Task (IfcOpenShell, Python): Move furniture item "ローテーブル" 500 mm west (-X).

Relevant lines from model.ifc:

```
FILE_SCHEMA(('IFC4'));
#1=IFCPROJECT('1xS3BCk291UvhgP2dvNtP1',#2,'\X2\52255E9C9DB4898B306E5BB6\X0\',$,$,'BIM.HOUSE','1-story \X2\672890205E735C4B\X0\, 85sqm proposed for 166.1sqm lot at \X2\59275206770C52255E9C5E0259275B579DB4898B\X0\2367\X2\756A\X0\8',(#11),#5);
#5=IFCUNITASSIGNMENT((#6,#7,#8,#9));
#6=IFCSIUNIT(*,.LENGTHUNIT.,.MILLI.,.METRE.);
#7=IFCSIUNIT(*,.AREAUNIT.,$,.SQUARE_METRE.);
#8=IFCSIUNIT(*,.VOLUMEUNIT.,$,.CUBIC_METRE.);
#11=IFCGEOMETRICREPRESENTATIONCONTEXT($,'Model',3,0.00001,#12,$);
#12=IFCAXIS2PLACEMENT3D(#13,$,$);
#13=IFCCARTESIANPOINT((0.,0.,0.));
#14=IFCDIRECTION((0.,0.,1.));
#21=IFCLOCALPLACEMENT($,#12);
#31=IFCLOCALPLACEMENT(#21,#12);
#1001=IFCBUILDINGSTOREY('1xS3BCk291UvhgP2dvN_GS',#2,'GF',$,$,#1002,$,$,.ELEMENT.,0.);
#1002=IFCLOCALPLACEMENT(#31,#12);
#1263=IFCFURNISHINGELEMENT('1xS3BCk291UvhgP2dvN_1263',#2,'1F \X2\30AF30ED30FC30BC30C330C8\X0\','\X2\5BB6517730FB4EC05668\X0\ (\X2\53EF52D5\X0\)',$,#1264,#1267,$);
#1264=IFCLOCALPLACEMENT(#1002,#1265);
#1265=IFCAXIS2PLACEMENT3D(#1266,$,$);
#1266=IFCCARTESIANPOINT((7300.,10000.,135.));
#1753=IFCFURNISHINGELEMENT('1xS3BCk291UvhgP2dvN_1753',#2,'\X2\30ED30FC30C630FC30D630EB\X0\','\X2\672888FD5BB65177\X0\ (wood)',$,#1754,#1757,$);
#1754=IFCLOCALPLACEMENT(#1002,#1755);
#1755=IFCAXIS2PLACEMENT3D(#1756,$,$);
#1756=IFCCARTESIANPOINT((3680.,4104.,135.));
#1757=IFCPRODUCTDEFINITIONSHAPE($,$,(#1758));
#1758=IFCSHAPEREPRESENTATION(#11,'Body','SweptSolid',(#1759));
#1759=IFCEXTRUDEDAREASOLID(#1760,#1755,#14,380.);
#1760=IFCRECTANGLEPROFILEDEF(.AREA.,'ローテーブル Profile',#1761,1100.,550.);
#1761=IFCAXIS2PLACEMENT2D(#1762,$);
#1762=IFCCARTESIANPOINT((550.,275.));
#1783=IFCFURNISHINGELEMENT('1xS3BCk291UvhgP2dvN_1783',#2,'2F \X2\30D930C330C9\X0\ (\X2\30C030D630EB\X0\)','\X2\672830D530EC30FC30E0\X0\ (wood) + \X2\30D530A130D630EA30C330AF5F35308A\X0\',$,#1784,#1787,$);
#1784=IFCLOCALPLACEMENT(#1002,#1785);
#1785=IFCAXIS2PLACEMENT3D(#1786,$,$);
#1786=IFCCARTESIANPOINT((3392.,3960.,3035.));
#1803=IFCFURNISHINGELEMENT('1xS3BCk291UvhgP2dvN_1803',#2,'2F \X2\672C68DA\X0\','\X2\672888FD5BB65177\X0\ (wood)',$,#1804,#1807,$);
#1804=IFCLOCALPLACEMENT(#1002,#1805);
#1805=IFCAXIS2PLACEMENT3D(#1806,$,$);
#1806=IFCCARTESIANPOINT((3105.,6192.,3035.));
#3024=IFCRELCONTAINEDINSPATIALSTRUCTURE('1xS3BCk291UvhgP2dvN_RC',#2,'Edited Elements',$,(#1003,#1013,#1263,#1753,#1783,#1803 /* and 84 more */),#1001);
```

```python
import ifcopenshell
import ifcopenshell.api.geometry
import ifcopenshell.util.placement

model = ifcopenshell.open("model.ifc")

item = model.by_guid("1xS3BCk291UvhgP2dvN_1753")
matrix = ifcopenshell.util.placement.get_local_placement(item.ObjectPlacement)
matrix[0, 3] -= 500.0
ifcopenshell.api.geometry.edit_object_placement(model, product=item, matrix=matrix, is_si=False)

print(ifcopenshell.util.placement.get_local_placement(item.ObjectPlacement).round(3) + 0.0)

model.write("model_rev.ifc")
```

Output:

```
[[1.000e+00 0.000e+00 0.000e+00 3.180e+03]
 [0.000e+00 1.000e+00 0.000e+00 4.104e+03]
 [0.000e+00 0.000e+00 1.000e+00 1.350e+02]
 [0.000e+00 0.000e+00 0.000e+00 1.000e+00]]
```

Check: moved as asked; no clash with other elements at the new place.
